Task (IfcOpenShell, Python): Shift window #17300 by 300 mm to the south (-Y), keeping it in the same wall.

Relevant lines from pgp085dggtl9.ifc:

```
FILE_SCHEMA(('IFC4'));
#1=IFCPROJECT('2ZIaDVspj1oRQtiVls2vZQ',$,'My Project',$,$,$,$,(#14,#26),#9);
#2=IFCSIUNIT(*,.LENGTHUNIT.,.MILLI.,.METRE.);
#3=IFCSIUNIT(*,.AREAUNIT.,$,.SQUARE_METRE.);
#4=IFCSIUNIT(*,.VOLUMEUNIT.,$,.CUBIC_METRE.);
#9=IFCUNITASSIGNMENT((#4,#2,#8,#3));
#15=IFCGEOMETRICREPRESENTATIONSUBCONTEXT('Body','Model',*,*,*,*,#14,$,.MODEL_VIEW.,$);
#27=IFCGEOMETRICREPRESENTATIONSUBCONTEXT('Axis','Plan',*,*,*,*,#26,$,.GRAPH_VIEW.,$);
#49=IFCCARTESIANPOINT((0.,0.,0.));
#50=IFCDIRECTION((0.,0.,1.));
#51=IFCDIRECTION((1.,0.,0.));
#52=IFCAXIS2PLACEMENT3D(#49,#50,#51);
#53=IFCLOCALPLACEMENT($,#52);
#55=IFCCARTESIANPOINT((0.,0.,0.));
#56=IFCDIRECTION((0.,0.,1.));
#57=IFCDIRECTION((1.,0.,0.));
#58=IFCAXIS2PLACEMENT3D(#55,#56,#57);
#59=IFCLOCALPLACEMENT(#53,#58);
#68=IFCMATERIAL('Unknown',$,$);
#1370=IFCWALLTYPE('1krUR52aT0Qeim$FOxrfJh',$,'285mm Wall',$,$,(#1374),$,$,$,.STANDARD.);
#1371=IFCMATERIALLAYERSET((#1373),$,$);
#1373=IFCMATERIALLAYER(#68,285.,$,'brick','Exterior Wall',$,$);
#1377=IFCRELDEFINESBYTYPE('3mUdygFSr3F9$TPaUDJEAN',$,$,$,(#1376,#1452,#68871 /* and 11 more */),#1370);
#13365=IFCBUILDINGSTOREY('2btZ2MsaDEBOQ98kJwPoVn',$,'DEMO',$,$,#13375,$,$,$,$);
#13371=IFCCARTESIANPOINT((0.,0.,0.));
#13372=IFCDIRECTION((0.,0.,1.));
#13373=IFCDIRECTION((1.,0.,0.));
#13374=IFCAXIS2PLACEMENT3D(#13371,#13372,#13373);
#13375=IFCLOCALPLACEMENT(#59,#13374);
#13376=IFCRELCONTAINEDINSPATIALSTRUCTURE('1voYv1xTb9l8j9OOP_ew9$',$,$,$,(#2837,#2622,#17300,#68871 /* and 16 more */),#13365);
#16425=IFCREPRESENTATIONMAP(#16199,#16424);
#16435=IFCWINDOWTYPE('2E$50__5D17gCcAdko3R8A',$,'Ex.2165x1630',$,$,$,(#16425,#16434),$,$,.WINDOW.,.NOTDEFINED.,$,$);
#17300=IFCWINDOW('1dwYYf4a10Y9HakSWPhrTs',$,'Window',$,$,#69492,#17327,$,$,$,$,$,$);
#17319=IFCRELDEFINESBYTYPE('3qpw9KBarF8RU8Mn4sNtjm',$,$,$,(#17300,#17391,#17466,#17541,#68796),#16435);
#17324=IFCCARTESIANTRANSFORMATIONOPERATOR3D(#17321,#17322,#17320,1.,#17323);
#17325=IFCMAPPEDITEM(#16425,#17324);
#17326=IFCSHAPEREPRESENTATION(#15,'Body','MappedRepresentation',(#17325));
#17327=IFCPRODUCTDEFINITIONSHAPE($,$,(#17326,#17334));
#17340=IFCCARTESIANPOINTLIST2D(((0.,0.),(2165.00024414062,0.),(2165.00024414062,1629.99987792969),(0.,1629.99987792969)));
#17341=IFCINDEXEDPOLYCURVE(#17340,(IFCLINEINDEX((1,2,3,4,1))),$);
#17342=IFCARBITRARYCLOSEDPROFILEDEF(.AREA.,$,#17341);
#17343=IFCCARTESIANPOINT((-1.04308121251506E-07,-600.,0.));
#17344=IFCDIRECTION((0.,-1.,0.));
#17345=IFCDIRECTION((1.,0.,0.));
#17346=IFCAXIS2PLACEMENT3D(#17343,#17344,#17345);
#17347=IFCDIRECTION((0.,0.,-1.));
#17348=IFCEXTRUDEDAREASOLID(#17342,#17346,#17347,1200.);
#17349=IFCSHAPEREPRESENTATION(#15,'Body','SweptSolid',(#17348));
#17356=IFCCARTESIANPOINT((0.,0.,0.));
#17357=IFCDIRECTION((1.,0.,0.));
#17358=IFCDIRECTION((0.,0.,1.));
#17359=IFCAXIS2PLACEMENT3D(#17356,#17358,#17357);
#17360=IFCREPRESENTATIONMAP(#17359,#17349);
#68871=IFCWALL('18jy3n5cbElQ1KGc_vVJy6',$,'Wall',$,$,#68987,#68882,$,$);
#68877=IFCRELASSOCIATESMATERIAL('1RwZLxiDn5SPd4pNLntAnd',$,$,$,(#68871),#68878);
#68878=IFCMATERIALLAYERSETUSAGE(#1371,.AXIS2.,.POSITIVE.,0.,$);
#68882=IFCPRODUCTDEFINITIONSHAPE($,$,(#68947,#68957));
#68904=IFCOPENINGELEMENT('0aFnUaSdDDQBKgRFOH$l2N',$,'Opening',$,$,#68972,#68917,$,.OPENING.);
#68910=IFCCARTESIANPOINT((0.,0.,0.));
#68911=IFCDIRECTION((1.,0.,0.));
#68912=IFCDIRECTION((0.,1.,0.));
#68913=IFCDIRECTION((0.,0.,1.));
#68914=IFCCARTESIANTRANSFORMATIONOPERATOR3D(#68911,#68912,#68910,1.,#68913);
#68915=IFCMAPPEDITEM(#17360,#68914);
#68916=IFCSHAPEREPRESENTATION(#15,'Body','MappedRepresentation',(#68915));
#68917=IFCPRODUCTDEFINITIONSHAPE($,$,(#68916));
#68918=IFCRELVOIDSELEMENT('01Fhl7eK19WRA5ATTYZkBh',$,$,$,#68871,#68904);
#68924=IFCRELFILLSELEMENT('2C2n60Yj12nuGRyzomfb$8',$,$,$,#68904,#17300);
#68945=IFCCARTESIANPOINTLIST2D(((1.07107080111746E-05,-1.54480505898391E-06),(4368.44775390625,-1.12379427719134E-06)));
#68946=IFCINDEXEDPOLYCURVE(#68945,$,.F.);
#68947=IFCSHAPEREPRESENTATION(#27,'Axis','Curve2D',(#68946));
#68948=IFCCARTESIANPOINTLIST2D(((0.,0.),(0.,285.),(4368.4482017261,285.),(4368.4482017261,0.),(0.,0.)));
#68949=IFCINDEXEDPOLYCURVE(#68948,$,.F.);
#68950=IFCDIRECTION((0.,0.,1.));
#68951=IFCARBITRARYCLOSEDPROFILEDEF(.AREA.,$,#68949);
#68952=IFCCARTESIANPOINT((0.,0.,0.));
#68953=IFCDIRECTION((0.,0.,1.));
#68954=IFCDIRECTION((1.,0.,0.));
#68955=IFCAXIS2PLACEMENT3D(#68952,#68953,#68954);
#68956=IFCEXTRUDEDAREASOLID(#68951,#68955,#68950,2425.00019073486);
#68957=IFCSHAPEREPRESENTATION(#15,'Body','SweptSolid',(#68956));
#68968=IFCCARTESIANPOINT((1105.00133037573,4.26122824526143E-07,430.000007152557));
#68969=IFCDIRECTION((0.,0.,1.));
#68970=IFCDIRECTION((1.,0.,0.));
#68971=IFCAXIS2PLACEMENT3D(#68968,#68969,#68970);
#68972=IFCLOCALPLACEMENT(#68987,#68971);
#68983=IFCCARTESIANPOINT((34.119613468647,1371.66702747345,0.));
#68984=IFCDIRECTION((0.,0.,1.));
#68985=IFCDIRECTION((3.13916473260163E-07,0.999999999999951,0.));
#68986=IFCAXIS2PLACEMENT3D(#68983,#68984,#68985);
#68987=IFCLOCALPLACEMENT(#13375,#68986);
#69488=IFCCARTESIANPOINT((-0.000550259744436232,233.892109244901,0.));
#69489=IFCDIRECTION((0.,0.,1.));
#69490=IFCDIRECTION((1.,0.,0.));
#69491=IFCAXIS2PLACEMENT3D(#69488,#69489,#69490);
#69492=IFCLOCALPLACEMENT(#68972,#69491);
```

```python
import ifcopenshell
import ifcopenshell.api.geometry
import ifcopenshell.util.placement

model = ifcopenshell.open("pgp085dggtl9.ifc")

window = model.by_id(17300)
opening = window.FillsVoids[0].RelatingOpeningElement
wall = opening.VoidsElements[0].RelatingBuildingElement

wall_matrix = ifcopenshell.util.placement.get_local_placement(wall.ObjectPlacement)
shift = wall_matrix[:3, 0] * -300.0
before = ifcopenshell.util.placement.get_local_placement(window.ObjectPlacement)[:3, 3].copy()

# The window is placed relative to its opening, so it follows when the opening moves.
matrix = ifcopenshell.util.placement.get_local_placement(opening.ObjectPlacement)
matrix[:3, 3] += shift
ifcopenshell.api.geometry.edit_object_placement(
    model, product=opening, matrix=matrix, is_si=False, should_transform_children=True
)

after = ifcopenshell.util.placement.get_local_placement(window.ObjectPlacement)[:3, 3]
print("window moved by", (after - before).round(3) + 0.0)

model.write("pgp085dggtl9_v2.ifc")
```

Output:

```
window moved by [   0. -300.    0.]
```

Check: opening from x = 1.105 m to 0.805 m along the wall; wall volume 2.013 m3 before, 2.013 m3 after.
